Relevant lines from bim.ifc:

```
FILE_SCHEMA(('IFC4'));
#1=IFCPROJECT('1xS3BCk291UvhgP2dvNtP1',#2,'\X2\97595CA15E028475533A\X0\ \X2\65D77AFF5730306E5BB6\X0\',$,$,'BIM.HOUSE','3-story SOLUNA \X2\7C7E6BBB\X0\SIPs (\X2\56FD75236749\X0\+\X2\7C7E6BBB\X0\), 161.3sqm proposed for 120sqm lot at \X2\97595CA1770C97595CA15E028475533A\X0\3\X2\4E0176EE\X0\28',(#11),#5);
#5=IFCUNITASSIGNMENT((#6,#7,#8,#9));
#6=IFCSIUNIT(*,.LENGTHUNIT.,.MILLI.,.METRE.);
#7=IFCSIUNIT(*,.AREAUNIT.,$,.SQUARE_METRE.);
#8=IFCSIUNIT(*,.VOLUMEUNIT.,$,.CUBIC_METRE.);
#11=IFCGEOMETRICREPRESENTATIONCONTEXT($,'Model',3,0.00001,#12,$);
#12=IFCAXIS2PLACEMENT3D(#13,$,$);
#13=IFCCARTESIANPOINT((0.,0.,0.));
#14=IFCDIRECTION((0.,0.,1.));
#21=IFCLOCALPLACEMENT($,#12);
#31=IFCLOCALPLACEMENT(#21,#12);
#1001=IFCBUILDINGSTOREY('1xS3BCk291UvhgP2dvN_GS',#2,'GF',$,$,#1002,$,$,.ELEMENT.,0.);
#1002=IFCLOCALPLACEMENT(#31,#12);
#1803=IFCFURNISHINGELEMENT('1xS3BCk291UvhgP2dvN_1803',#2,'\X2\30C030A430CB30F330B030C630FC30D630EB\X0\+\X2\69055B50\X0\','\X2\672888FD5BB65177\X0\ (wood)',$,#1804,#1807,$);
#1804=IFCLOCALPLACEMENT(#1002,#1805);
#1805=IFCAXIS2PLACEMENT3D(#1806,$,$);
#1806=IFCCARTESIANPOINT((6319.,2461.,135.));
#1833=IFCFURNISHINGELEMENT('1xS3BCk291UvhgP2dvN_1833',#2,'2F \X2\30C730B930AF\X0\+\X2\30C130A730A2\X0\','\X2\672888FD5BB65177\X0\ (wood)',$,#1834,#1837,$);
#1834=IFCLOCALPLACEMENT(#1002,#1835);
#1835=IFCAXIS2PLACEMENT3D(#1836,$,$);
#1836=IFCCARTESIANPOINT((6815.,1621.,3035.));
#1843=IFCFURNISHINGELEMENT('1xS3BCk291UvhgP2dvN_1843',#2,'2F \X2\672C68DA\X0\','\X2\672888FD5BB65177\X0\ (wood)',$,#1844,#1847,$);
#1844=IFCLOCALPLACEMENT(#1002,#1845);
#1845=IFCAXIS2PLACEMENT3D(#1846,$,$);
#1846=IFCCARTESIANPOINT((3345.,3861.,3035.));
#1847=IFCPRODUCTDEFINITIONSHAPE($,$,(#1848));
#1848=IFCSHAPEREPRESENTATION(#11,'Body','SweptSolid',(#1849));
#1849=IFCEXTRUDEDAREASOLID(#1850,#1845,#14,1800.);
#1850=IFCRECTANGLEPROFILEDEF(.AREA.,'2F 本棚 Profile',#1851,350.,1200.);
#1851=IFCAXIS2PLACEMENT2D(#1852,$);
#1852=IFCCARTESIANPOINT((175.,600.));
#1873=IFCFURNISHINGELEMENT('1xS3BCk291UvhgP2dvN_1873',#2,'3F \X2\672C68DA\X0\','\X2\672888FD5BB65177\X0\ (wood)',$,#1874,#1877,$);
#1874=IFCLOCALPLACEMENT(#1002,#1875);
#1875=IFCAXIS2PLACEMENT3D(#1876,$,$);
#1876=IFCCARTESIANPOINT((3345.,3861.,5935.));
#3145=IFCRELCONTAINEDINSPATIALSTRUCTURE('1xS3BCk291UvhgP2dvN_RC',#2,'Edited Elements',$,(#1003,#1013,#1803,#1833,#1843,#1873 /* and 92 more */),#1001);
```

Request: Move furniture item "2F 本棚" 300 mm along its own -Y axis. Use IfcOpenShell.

```python
import ifcopenshell
import ifcopenshell.api.geometry
import ifcopenshell.util.placement

model = ifcopenshell.open("bim.ifc")

item = model.by_id(1843)
matrix = ifcopenshell.util.placement.get_local_placement(item.ObjectPlacement)
matrix[:3, 3] -= matrix[:3, 1] * 300.0
ifcopenshell.api.geometry.edit_object_placement(model, product=item, matrix=matrix, is_si=False)

print(ifcopenshell.util.placement.get_local_placement(item.ObjectPlacement).round(3) + 0.0)

model.write("bim_rev.ifc")
```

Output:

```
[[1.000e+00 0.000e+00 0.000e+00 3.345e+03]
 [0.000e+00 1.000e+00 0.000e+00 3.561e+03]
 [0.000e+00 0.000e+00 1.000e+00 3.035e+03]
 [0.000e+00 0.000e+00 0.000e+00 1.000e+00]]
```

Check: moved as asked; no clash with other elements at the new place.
